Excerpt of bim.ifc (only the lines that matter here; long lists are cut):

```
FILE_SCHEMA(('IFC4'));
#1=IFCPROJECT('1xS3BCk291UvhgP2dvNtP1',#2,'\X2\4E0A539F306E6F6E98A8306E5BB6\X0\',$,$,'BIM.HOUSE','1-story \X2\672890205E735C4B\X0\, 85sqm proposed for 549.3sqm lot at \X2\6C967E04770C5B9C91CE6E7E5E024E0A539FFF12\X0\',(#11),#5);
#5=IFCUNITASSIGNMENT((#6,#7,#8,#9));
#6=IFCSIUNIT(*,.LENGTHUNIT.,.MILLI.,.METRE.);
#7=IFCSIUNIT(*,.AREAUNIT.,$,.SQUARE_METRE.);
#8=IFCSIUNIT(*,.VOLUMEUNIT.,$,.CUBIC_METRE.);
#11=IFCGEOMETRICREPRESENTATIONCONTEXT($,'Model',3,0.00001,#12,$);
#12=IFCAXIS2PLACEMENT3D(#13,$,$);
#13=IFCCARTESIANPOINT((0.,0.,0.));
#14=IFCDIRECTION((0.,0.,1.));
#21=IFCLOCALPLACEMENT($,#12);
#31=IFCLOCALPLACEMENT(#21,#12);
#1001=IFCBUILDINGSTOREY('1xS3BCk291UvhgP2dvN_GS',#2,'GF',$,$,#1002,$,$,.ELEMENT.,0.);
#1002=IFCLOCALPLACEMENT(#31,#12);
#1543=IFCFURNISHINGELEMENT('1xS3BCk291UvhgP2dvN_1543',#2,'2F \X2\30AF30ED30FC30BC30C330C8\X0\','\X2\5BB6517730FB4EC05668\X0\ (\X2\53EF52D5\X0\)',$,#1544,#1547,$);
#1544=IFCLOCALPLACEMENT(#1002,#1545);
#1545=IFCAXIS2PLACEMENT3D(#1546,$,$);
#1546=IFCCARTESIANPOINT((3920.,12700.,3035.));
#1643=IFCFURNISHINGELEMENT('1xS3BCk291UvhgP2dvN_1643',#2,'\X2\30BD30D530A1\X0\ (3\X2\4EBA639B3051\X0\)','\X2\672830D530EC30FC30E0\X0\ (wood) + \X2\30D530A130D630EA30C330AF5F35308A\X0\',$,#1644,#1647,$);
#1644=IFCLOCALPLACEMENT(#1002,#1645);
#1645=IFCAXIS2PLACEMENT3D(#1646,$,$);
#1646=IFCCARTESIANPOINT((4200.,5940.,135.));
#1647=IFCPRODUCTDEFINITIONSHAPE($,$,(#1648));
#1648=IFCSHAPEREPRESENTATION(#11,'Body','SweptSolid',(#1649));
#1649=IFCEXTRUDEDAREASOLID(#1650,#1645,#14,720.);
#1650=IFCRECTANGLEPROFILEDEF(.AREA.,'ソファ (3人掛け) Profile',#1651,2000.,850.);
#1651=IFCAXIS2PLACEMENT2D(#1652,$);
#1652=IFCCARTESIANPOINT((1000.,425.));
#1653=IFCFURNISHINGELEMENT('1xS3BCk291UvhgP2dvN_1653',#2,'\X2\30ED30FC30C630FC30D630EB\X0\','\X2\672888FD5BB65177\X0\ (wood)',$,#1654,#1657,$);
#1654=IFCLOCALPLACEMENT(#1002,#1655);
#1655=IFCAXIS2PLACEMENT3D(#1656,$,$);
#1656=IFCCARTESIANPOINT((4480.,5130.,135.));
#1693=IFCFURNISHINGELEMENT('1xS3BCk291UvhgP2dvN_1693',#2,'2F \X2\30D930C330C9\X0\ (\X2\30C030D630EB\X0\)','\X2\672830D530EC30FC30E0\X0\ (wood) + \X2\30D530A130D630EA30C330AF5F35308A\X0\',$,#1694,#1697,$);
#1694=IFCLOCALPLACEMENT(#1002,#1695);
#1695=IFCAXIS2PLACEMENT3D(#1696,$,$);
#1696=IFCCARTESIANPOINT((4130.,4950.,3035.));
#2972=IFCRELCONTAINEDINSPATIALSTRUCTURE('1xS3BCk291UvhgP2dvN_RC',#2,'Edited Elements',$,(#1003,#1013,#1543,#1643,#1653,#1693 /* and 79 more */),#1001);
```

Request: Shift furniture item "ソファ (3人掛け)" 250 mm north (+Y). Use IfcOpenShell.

```python
import ifcopenshell
import ifcopenshell.api.geometry
import ifcopenshell.util.placement
import ifcopenshell.util.unit

model = ifcopenshell.open("bim.ifc")
unit_scale = ifcopenshell.util.unit.calculate_unit_scale(model)

item = model.by_guid("1xS3BCk291UvhgP2dvN_1643")
matrix = ifcopenshell.util.placement.get_local_placement(item.ObjectPlacement)
matrix[1, 3] += 0.25 / unit_scale
ifcopenshell.api.geometry.edit_object_placement(model, product=item, matrix=matrix, is_si=False)

print(ifcopenshell.util.placement.get_local_placement(item.ObjectPlacement).round(3) + 0.0)

model.write("bim_updated.ifc")
```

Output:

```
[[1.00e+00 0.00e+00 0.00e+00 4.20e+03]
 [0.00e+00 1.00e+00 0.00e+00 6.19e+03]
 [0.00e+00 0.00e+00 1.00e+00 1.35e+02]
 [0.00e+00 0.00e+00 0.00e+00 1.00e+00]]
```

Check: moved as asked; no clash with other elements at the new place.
